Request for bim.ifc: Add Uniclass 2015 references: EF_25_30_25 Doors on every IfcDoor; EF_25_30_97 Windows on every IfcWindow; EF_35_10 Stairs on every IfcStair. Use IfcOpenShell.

First a look at what the model holds.

```python
import ifcopenshell

model = ifcopenshell.open("bim.ifc")
print(model.schema)
print("classifications:", [c.Name for c in model.by_type("IfcClassification")])
for ifc_class in ("IfcDoor", "IfcRoof", "IfcStair", "IfcWall", "IfcWindow"):
    print(ifc_class, len(model.by_type(ifc_class)))
```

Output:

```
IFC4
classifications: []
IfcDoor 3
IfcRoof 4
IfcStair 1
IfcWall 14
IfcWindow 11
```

```python
import ifcopenshell
import ifcopenshell.api.classification

model = ifcopenshell.open("bim.ifc")

system = ifcopenshell.api.classification.add_classification(model, classification="Uniclass 2015")

codes = {
    "IfcDoor": ("EF_25_30_25", "Doors"),
    "IfcWindow": ("EF_25_30_97", "Windows"),
    "IfcStair": ("EF_35_10", "Stairs"),
}
for ifc_class, (code, name) in codes.items():
    products = model.by_type(ifc_class)
    ifcopenshell.api.classification.add_reference(
        model, products=products, classification=system, identification=code, name=name
    )
    print(code, len(products))

model.write("bim-out.ifc")
```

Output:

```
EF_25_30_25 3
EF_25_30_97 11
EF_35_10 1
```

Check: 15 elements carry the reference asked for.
